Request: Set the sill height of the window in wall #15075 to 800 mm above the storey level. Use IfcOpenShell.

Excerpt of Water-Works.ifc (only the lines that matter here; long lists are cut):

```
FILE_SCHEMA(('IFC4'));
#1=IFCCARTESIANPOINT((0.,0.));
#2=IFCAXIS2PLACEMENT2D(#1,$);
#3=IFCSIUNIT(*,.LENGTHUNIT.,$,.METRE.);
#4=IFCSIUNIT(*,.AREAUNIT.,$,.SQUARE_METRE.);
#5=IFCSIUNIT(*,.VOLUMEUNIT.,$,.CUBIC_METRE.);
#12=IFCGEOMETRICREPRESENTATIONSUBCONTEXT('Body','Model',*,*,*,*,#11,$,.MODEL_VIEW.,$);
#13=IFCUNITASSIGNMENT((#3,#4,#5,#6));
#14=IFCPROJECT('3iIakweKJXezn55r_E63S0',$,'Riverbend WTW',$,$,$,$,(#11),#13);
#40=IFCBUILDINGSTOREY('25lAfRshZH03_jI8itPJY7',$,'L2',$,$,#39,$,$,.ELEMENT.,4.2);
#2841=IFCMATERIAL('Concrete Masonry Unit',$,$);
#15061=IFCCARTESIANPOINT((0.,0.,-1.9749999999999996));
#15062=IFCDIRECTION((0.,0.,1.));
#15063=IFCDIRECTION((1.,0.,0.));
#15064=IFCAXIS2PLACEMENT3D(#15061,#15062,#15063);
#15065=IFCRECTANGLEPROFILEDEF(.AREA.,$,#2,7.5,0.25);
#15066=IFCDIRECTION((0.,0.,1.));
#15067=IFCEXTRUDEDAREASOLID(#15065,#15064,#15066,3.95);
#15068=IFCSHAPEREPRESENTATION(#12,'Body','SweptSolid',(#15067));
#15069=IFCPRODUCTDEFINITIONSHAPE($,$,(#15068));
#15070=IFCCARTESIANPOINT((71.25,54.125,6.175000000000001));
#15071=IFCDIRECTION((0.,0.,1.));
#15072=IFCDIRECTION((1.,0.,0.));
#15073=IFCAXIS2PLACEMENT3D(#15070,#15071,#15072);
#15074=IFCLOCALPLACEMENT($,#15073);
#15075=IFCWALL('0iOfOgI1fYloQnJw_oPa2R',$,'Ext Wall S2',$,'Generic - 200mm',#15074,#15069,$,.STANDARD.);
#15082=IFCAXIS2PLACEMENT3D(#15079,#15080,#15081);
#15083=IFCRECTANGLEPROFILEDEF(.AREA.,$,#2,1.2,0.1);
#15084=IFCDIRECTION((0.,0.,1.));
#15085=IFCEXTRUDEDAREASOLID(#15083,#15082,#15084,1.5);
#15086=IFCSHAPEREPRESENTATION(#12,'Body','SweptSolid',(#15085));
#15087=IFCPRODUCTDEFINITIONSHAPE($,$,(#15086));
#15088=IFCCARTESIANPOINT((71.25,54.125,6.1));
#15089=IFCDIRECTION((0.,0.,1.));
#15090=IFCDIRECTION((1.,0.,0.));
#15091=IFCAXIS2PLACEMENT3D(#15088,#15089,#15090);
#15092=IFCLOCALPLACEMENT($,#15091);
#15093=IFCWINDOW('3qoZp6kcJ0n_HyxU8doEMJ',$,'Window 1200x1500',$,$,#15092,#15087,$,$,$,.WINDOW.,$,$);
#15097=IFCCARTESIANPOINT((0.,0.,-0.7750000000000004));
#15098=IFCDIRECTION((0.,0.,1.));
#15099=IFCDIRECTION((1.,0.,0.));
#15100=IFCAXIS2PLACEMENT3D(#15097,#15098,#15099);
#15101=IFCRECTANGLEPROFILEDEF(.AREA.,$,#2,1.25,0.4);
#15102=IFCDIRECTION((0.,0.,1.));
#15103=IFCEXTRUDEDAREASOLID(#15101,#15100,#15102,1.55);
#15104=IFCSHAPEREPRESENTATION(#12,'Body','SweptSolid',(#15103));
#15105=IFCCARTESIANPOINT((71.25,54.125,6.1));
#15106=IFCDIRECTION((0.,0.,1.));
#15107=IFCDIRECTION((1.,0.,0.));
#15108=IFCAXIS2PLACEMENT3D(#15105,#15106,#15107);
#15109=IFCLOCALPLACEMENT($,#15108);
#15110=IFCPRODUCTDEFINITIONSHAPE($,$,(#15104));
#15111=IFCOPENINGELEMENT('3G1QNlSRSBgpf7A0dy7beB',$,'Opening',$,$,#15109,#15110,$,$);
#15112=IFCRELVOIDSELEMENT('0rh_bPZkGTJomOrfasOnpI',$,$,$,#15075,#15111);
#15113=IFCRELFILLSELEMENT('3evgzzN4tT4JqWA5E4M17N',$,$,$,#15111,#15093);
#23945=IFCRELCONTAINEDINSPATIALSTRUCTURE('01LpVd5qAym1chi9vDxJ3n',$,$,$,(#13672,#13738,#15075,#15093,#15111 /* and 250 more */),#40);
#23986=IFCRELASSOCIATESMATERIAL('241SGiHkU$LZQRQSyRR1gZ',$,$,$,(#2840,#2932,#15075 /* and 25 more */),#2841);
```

```python
import numpy as np
import ifcopenshell
import ifcopenshell.api.geometry
import ifcopenshell.geom
import ifcopenshell.util.element
import ifcopenshell.util.placement
import ifcopenshell.util.shape
import ifcopenshell.util.unit

model = ifcopenshell.open("Water-Works.ifc")
unit_scale = ifcopenshell.util.unit.calculate_unit_scale(model)

window = model.by_guid("3qoZp6kcJ0n_HyxU8doEMJ")
opening = window.FillsVoids[0].RelatingOpeningElement
storey = ifcopenshell.util.element.get_container(window, ifc_class="IfcBuildingStorey")
level = ifcopenshell.util.placement.get_local_placement(storey.ObjectPlacement)[2, 3]

# The opening's origin need not be at the sill, so measure its lowest point.
shape = ifcopenshell.geom.create_shape(ifcopenshell.geom.settings(), opening)
bottom = ifcopenshell.util.shape.get_shape_bottom_elevation(shape, shape.geometry) / unit_scale
dz = level + 0.8 / unit_scale - bottom

shift = np.array([0.0, 0.0, dz])
# The window is not placed relative to its opening, so move both.
for product in (opening, window):
    matrix = ifcopenshell.util.placement.get_local_placement(product.ObjectPlacement)
    matrix[:3, 3] += shift
    ifcopenshell.api.geometry.edit_object_placement(model, product=product, matrix=matrix, is_si=False)

print(f"moved by {dz * unit_scale:+.3f} m")

model.write("Water-Works-out.ifc")
```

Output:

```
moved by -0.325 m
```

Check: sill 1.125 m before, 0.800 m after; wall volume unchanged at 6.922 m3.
